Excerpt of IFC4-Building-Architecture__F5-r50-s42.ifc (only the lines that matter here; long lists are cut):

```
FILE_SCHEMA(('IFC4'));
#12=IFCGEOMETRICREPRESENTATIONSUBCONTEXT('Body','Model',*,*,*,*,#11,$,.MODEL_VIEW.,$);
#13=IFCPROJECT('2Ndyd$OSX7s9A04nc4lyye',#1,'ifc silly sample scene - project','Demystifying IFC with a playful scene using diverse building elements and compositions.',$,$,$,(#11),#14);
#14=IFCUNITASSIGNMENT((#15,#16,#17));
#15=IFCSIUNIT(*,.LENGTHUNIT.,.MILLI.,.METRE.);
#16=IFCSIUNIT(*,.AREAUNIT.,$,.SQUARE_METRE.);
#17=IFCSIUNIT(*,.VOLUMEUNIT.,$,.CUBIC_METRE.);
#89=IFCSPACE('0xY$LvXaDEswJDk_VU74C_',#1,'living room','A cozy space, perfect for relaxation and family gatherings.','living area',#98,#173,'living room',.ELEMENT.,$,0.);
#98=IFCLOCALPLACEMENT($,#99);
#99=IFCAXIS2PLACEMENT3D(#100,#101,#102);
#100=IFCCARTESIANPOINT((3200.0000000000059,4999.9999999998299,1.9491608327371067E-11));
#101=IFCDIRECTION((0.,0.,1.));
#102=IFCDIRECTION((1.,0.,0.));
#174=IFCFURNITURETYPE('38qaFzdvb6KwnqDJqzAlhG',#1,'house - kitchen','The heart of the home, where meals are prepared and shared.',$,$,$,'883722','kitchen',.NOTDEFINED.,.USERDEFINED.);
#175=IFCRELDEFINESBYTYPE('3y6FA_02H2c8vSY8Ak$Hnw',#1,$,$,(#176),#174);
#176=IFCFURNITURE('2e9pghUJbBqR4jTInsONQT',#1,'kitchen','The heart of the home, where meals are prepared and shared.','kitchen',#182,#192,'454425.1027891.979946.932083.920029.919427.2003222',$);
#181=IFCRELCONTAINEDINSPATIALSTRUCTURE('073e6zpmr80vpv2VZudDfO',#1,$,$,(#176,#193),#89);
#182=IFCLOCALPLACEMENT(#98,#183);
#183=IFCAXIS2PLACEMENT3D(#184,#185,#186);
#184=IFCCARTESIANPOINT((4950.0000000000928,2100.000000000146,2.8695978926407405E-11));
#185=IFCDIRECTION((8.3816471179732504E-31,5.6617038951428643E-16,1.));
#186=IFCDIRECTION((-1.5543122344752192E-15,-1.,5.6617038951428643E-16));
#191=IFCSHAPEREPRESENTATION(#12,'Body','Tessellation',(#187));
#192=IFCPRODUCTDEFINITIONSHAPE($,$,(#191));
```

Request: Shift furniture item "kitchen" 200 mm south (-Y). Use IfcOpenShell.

```python
import ifcopenshell
import ifcopenshell.api.geometry
import ifcopenshell.util.placement
import ifcopenshell.util.unit

model = ifcopenshell.open("IFC4-Building-Architecture__F5-r50-s42.ifc")
unit_scale = ifcopenshell.util.unit.calculate_unit_scale(model)

item = model.by_id(176)
matrix = ifcopenshell.util.placement.get_local_placement(item.ObjectPlacement)
matrix[1, 3] -= 0.2 / unit_scale
ifcopenshell.api.geometry.edit_object_placement(model, product=item, matrix=matrix, is_si=False)

print(ifcopenshell.util.placement.get_local_placement(item.ObjectPlacement).round(3) + 0.0)

model.write("IFC4-Building-Architecture__F5-r50-s42_rev.ifc")
```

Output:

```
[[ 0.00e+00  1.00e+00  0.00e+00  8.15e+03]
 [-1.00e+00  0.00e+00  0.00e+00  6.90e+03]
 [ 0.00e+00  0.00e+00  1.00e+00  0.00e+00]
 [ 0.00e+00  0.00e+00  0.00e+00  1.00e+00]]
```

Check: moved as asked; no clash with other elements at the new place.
